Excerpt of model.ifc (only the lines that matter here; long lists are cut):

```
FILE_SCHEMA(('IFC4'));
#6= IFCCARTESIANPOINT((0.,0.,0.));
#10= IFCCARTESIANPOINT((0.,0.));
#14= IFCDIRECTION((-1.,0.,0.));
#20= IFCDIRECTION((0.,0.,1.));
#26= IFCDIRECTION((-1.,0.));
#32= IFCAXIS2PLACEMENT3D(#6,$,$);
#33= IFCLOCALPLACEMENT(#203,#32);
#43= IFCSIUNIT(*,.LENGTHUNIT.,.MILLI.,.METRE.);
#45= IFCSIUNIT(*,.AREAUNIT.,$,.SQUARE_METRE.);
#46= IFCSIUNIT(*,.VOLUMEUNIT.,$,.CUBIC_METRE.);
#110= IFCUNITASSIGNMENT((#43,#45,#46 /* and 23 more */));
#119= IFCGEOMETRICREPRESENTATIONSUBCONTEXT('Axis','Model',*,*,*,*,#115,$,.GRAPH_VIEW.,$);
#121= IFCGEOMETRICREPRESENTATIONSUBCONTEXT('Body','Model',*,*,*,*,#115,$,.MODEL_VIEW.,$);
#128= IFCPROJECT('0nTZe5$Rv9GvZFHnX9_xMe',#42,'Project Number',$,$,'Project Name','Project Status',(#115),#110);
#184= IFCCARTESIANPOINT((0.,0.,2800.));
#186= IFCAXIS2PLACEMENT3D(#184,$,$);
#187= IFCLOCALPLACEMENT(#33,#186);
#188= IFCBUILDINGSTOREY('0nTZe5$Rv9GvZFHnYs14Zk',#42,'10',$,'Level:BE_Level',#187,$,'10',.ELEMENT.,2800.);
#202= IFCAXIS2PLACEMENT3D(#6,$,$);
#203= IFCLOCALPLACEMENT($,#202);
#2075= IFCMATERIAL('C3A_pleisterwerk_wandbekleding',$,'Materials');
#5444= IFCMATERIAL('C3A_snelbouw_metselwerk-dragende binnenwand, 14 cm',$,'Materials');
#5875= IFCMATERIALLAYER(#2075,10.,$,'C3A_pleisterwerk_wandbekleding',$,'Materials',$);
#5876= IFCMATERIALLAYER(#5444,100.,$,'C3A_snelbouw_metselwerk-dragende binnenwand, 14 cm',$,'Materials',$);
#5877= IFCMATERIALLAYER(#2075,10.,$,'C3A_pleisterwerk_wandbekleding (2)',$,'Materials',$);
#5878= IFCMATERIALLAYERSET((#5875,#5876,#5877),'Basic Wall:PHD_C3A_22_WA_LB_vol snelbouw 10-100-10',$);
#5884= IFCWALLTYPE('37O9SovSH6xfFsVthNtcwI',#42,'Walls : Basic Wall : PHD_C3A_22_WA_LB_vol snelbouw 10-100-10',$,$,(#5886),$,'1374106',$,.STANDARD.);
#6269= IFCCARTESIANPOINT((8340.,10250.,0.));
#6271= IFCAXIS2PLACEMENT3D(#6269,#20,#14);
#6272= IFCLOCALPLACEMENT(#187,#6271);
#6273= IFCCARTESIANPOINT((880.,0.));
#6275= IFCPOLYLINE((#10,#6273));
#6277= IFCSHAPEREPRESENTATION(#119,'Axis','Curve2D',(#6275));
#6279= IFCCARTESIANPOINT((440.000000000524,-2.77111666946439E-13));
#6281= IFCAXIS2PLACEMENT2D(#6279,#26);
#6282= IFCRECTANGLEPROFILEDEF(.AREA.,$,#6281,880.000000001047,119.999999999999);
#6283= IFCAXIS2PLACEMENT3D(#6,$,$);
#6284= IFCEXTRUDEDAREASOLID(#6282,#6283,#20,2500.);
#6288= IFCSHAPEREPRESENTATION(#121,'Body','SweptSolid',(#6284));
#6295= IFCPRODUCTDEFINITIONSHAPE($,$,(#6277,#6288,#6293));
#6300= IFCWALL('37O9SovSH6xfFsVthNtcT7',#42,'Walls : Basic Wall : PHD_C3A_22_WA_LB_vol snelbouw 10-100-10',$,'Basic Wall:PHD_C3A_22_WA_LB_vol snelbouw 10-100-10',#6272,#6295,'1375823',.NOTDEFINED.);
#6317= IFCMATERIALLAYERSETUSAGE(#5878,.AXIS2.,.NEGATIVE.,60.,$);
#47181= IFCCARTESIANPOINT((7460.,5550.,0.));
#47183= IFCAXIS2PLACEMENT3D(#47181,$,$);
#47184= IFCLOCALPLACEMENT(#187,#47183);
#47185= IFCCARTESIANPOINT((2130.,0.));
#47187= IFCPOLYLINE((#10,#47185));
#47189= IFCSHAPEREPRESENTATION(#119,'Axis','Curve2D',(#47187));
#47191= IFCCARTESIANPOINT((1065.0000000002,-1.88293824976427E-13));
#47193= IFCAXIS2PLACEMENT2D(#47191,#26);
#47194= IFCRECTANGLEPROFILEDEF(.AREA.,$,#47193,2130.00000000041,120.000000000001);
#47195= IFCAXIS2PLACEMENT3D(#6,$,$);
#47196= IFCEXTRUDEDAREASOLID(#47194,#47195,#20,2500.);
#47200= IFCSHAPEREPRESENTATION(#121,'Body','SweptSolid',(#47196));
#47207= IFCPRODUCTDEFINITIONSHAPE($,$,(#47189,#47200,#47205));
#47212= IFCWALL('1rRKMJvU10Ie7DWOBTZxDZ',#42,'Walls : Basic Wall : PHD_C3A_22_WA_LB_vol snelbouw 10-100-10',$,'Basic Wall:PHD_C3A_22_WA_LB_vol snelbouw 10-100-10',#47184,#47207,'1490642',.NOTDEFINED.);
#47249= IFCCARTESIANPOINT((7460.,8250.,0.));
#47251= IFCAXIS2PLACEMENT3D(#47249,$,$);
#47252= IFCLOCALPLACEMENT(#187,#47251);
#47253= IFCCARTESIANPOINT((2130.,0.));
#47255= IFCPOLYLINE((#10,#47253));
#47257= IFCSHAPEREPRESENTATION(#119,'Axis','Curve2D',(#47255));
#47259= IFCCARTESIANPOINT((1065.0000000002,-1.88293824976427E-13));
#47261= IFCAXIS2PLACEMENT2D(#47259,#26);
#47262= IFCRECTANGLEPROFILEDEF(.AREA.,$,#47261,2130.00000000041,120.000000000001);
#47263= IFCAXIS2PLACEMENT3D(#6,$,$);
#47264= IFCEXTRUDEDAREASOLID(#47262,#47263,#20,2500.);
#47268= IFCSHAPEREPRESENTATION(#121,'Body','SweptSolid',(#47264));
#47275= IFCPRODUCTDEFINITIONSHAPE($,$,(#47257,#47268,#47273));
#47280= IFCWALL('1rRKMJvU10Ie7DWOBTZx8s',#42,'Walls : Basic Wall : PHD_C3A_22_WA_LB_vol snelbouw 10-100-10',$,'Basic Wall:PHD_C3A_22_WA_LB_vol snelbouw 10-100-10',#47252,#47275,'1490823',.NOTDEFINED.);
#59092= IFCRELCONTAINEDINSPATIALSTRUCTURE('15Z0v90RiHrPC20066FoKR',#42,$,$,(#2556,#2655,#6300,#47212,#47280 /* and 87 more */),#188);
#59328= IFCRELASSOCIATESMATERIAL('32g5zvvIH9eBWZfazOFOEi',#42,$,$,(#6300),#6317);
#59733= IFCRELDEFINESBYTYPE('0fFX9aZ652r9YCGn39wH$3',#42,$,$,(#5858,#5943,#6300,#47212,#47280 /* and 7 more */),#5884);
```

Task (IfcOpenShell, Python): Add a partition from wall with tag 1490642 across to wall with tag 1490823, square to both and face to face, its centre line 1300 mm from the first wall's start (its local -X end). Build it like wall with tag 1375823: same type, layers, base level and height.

```python
import numpy as np
import ifcopenshell
import ifcopenshell.api.geometry
import ifcopenshell.api.material
import ifcopenshell.api.pset
import ifcopenshell.api.root
import ifcopenshell.api.spatial
import ifcopenshell.api.type
import ifcopenshell.geom
import ifcopenshell.util.element
import ifcopenshell.util.placement
import ifcopenshell.util.representation
import ifcopenshell.util.shape
import ifcopenshell.util.unit

model = ifcopenshell.open("model.ifc")
unit_scale = ifcopenshell.util.unit.calculate_unit_scale(model)
settings = ifcopenshell.geom.settings()
settings.set("use-world-coords", True)

start_wall = model.by_guid("1rRKMJvU10Ie7DWOBTZxDZ")
end_wall = model.by_guid("1rRKMJvU10Ie7DWOBTZx8s")
like = model.by_guid("37O9SovSH6xfFsVthNtcT7")
matrix = ifcopenshell.util.placement.get_local_placement(start_wall.ObjectPlacement)
matrix[:3, 3] *= unit_scale


def extent(element):
    """Bounding box in the first wall's axes, in metres."""
    shape = ifcopenshell.geom.create_shape(settings, element)
    points = (ifcopenshell.util.shape.get_vertices(shape.geometry) - matrix[:3, 3]) @ matrix[:3, :3]
    return points.min(axis=0), points.max(axis=0)


y_start = extent(start_wall)[1][1]
y_end = extent(end_wall)[0][1]
like_min, like_max = extent(like)
length, height = float(abs(y_end - y_start)), float(like_max[2] - like_min[2])
layer_set = ifcopenshell.util.element.get_material(like, should_skip_usage=True)
thickness = sum(layer.LayerThickness for layer in layer_set.MaterialLayers) * unit_scale

wall = ifcopenshell.api.root.create_entity(model, ifc_class="IfcWall", name="New partition")
storey = ifcopenshell.util.element.get_container(like)
ifcopenshell.api.spatial.assign_container(model, products=[wall], relating_structure=storey)
ifcopenshell.api.type.assign_type(
    model, related_objects=[wall], relating_type=ifcopenshell.util.element.get_type(like), should_map_representations=False
)
rel = ifcopenshell.api.material.assign_material(
    model, products=[wall], type="IfcMaterialLayerSetUsage", material=layer_set
)
rel.RelatingMaterial.OffsetFromReferenceLine = -thickness / 2 / unit_scale
pset = ifcopenshell.api.pset.add_pset(model, product=wall, name="Pset_WallCommon")
ifcopenshell.api.pset.edit_pset(model, pset=pset, properties={"IsExternal": False, "LoadBearing": False})

# The axis runs down the middle of the wall.
axis = ifcopenshell.api.geometry.add_axis_representation(
    model, context=ifcopenshell.util.representation.get_context(model, "Model", "Axis"), axis=[(0.0, 0.0), (length, 0.0)]
)
body = ifcopenshell.api.geometry.add_wall_representation(
    model,
    context=ifcopenshell.util.representation.get_context(model, "Model", "Body", "MODEL_VIEW"),
    length=length,
    height=height,
    thickness=thickness,
    offset=-thickness / 2,
)
for representation in (axis, body):
    ifcopenshell.api.geometry.assign_representation(model, product=wall, representation=representation)

placement = matrix @ ifcopenshell.util.placement.rotation(90, "Z")
placement[:, 3] = matrix @ np.array([extent(start_wall)[0][0] + 1.3, y_start, like_min[2], 1.0])
ifcopenshell.api.geometry.edit_object_placement(model, product=wall, matrix=placement)

print(f"partition {length:.3f} m long, {height:.3f} m high, {thickness:.3f} m thick")

model.write("model_v2.ifc")
```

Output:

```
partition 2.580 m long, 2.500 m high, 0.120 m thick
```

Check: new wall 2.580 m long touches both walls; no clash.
